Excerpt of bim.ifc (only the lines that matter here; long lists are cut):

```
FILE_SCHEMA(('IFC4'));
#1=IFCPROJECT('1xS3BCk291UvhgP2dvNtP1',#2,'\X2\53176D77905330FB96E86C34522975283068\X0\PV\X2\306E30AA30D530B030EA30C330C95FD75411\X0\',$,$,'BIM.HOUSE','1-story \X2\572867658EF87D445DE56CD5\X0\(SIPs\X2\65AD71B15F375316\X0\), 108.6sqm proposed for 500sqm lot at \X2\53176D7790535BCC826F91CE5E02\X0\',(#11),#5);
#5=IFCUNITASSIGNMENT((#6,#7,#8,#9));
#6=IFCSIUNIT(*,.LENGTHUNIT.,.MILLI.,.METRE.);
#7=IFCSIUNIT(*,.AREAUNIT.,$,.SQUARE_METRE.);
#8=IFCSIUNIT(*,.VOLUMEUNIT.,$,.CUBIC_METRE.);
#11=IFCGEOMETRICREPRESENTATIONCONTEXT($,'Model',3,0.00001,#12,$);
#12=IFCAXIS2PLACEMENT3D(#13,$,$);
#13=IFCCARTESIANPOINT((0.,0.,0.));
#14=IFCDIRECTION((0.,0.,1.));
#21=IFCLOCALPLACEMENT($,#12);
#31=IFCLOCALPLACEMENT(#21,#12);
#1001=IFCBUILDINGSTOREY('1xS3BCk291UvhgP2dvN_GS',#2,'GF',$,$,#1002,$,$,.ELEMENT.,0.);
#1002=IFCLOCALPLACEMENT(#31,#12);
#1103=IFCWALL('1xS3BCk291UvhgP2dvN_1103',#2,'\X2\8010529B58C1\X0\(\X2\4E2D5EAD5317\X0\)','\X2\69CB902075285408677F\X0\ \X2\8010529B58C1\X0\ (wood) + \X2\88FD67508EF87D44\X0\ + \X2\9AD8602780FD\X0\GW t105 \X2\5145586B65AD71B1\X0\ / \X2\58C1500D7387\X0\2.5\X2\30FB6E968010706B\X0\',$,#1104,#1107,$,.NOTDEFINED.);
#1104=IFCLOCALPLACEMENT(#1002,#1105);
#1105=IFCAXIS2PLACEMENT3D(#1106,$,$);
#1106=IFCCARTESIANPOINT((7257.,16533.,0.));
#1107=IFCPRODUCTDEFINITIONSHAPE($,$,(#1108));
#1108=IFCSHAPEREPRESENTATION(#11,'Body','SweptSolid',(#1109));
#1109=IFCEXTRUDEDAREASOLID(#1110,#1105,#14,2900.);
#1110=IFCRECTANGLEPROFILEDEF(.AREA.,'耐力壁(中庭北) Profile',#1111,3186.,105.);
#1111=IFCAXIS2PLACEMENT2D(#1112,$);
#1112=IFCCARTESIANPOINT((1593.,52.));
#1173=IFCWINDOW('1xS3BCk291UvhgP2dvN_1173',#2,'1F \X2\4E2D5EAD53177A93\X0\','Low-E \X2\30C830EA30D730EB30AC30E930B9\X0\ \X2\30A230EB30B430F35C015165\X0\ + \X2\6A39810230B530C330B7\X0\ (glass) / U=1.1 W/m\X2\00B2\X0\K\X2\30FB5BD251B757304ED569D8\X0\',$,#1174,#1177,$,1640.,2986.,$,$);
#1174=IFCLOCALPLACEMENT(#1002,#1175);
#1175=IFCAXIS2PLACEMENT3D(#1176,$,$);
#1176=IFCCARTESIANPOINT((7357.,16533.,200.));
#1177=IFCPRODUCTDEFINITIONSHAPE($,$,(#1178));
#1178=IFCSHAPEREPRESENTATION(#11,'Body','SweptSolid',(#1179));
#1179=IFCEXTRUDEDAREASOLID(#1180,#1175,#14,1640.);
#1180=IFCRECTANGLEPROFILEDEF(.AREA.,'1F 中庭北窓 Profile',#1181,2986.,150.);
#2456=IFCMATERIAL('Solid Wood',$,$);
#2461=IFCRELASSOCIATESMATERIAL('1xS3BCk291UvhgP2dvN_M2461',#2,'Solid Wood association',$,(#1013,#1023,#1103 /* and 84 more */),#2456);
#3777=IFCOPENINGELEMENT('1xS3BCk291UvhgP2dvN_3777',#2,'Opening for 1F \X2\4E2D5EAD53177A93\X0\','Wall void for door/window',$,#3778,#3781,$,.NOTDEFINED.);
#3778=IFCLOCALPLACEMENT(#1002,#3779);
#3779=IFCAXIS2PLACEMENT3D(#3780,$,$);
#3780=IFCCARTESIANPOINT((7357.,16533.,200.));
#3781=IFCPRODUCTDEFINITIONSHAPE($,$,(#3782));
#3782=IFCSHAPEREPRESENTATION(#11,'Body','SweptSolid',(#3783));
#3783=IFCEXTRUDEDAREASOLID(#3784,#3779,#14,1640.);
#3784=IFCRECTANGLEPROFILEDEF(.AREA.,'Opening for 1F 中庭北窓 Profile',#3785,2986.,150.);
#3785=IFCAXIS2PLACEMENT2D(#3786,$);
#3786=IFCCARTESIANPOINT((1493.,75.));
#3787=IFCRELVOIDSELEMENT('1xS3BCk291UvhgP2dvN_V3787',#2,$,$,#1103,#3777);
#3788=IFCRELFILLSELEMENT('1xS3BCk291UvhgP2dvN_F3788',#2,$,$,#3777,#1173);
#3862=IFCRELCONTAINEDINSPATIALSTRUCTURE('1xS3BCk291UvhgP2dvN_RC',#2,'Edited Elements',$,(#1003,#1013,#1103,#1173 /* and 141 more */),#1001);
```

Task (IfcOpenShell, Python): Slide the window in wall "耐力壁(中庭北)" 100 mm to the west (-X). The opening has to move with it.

```python
import ifcopenshell
import ifcopenshell.api.geometry
import ifcopenshell.util.placement
import ifcopenshell.util.unit

model = ifcopenshell.open("bim.ifc")
unit_scale = ifcopenshell.util.unit.calculate_unit_scale(model)

window = model.by_id(1173)
opening = window.FillsVoids[0].RelatingOpeningElement
wall = opening.VoidsElements[0].RelatingBuildingElement

wall_matrix = ifcopenshell.util.placement.get_local_placement(wall.ObjectPlacement)
shift = wall_matrix[:3, 0] * -0.1 / unit_scale
before = ifcopenshell.util.placement.get_local_placement(window.ObjectPlacement)[:3, 3].copy()

# The window is not placed relative to its opening, so move both.
for product in (opening, window):
    matrix = ifcopenshell.util.placement.get_local_placement(product.ObjectPlacement)
    matrix[:3, 3] += shift
    ifcopenshell.api.geometry.edit_object_placement(model, product=product, matrix=matrix, is_si=False)

after = ifcopenshell.util.placement.get_local_placement(window.ObjectPlacement)[:3, 3]
print("window moved by", (after - before).round(3) + 0.0)

model.write("bim-out.ifc")
```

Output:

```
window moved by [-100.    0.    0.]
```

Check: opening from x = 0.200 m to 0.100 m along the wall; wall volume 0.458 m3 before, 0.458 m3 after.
